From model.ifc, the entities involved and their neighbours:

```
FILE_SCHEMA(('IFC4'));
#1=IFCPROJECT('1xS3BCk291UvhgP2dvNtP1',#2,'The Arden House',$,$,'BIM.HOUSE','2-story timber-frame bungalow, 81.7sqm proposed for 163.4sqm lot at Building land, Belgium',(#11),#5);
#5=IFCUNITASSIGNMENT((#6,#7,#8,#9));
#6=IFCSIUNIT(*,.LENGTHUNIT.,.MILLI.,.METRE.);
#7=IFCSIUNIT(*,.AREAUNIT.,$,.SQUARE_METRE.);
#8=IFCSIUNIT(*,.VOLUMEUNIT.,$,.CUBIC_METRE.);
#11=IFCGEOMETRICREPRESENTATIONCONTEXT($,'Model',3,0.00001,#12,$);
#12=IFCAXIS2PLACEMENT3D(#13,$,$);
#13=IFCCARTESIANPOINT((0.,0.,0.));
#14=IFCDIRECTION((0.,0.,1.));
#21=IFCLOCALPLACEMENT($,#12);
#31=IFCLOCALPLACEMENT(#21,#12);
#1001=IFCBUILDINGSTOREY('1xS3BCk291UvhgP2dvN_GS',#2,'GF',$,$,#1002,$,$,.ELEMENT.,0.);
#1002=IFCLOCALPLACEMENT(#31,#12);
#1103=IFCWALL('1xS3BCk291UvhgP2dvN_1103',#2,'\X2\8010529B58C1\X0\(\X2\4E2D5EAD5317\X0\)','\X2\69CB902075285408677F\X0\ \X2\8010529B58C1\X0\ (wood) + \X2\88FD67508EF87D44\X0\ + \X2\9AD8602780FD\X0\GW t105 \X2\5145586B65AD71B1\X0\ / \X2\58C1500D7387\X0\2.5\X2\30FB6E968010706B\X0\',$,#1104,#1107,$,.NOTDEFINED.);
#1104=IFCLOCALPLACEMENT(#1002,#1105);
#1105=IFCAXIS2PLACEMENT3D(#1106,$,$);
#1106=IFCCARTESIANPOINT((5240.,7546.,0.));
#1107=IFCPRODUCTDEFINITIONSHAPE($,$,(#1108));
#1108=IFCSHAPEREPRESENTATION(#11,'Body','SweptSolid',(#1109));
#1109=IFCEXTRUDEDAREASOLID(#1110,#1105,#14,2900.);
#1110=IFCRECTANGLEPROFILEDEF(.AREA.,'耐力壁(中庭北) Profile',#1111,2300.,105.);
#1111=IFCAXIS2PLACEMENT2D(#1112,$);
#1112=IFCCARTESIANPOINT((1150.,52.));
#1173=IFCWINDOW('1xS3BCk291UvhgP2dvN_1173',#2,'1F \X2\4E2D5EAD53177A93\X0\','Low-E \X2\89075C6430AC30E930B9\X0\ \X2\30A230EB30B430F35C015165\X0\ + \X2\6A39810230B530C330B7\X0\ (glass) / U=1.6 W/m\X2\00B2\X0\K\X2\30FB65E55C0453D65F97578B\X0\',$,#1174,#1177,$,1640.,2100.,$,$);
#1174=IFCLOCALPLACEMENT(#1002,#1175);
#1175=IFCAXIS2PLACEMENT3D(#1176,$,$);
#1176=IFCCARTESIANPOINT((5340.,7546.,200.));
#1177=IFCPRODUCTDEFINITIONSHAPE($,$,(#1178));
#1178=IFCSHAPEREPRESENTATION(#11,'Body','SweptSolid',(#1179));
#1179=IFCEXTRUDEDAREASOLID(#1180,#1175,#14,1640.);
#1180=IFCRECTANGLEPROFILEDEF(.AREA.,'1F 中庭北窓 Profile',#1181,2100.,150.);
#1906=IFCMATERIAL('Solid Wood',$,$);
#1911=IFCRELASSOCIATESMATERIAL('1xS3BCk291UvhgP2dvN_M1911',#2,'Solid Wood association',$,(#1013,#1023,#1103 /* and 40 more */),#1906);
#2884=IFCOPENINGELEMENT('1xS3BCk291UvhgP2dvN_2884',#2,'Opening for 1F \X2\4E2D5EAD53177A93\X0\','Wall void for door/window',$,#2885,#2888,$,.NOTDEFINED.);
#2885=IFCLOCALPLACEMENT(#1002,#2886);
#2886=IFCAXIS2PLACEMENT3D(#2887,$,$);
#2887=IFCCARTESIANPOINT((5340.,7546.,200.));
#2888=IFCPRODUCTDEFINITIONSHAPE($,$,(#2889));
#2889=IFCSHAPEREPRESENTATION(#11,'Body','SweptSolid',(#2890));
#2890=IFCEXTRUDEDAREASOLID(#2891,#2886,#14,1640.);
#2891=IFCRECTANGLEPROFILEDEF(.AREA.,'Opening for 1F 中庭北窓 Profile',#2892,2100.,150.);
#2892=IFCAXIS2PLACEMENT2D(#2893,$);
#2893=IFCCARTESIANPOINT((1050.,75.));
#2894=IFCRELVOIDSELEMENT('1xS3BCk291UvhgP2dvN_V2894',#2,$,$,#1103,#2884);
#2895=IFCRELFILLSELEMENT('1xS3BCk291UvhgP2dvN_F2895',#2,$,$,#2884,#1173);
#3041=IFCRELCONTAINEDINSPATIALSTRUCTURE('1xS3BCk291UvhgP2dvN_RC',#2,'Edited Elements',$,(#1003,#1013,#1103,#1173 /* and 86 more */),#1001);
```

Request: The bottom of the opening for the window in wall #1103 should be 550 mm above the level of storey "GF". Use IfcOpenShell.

```python
import numpy as np
import ifcopenshell
import ifcopenshell.api.geometry
import ifcopenshell.geom
import ifcopenshell.util.element
import ifcopenshell.util.placement
import ifcopenshell.util.shape
import ifcopenshell.util.unit

model = ifcopenshell.open("model.ifc")
unit_scale = ifcopenshell.util.unit.calculate_unit_scale(model)

window = model.by_id(1173)
opening = window.FillsVoids[0].RelatingOpeningElement
storey = ifcopenshell.util.element.get_container(window, ifc_class="IfcBuildingStorey")
level = ifcopenshell.util.placement.get_local_placement(storey.ObjectPlacement)[2, 3]

# The opening's origin need not be at the sill, so measure its lowest point.
shape = ifcopenshell.geom.create_shape(ifcopenshell.geom.settings(), opening)
bottom = ifcopenshell.util.shape.get_shape_bottom_elevation(shape, shape.geometry) / unit_scale
dz = level + 550.0 - bottom

shift = np.array([0.0, 0.0, dz])
# The window is not placed relative to its opening, so move both.
for product in (opening, window):
    matrix = ifcopenshell.util.placement.get_local_placement(product.ObjectPlacement)
    matrix[:3, 3] += shift
    ifcopenshell.api.geometry.edit_object_placement(model, product=product, matrix=matrix, is_si=False)

print(f"moved by {dz * unit_scale:+.3f} m")

model.write("model_updated.ifc")
```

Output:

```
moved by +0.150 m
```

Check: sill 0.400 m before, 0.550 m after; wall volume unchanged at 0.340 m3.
